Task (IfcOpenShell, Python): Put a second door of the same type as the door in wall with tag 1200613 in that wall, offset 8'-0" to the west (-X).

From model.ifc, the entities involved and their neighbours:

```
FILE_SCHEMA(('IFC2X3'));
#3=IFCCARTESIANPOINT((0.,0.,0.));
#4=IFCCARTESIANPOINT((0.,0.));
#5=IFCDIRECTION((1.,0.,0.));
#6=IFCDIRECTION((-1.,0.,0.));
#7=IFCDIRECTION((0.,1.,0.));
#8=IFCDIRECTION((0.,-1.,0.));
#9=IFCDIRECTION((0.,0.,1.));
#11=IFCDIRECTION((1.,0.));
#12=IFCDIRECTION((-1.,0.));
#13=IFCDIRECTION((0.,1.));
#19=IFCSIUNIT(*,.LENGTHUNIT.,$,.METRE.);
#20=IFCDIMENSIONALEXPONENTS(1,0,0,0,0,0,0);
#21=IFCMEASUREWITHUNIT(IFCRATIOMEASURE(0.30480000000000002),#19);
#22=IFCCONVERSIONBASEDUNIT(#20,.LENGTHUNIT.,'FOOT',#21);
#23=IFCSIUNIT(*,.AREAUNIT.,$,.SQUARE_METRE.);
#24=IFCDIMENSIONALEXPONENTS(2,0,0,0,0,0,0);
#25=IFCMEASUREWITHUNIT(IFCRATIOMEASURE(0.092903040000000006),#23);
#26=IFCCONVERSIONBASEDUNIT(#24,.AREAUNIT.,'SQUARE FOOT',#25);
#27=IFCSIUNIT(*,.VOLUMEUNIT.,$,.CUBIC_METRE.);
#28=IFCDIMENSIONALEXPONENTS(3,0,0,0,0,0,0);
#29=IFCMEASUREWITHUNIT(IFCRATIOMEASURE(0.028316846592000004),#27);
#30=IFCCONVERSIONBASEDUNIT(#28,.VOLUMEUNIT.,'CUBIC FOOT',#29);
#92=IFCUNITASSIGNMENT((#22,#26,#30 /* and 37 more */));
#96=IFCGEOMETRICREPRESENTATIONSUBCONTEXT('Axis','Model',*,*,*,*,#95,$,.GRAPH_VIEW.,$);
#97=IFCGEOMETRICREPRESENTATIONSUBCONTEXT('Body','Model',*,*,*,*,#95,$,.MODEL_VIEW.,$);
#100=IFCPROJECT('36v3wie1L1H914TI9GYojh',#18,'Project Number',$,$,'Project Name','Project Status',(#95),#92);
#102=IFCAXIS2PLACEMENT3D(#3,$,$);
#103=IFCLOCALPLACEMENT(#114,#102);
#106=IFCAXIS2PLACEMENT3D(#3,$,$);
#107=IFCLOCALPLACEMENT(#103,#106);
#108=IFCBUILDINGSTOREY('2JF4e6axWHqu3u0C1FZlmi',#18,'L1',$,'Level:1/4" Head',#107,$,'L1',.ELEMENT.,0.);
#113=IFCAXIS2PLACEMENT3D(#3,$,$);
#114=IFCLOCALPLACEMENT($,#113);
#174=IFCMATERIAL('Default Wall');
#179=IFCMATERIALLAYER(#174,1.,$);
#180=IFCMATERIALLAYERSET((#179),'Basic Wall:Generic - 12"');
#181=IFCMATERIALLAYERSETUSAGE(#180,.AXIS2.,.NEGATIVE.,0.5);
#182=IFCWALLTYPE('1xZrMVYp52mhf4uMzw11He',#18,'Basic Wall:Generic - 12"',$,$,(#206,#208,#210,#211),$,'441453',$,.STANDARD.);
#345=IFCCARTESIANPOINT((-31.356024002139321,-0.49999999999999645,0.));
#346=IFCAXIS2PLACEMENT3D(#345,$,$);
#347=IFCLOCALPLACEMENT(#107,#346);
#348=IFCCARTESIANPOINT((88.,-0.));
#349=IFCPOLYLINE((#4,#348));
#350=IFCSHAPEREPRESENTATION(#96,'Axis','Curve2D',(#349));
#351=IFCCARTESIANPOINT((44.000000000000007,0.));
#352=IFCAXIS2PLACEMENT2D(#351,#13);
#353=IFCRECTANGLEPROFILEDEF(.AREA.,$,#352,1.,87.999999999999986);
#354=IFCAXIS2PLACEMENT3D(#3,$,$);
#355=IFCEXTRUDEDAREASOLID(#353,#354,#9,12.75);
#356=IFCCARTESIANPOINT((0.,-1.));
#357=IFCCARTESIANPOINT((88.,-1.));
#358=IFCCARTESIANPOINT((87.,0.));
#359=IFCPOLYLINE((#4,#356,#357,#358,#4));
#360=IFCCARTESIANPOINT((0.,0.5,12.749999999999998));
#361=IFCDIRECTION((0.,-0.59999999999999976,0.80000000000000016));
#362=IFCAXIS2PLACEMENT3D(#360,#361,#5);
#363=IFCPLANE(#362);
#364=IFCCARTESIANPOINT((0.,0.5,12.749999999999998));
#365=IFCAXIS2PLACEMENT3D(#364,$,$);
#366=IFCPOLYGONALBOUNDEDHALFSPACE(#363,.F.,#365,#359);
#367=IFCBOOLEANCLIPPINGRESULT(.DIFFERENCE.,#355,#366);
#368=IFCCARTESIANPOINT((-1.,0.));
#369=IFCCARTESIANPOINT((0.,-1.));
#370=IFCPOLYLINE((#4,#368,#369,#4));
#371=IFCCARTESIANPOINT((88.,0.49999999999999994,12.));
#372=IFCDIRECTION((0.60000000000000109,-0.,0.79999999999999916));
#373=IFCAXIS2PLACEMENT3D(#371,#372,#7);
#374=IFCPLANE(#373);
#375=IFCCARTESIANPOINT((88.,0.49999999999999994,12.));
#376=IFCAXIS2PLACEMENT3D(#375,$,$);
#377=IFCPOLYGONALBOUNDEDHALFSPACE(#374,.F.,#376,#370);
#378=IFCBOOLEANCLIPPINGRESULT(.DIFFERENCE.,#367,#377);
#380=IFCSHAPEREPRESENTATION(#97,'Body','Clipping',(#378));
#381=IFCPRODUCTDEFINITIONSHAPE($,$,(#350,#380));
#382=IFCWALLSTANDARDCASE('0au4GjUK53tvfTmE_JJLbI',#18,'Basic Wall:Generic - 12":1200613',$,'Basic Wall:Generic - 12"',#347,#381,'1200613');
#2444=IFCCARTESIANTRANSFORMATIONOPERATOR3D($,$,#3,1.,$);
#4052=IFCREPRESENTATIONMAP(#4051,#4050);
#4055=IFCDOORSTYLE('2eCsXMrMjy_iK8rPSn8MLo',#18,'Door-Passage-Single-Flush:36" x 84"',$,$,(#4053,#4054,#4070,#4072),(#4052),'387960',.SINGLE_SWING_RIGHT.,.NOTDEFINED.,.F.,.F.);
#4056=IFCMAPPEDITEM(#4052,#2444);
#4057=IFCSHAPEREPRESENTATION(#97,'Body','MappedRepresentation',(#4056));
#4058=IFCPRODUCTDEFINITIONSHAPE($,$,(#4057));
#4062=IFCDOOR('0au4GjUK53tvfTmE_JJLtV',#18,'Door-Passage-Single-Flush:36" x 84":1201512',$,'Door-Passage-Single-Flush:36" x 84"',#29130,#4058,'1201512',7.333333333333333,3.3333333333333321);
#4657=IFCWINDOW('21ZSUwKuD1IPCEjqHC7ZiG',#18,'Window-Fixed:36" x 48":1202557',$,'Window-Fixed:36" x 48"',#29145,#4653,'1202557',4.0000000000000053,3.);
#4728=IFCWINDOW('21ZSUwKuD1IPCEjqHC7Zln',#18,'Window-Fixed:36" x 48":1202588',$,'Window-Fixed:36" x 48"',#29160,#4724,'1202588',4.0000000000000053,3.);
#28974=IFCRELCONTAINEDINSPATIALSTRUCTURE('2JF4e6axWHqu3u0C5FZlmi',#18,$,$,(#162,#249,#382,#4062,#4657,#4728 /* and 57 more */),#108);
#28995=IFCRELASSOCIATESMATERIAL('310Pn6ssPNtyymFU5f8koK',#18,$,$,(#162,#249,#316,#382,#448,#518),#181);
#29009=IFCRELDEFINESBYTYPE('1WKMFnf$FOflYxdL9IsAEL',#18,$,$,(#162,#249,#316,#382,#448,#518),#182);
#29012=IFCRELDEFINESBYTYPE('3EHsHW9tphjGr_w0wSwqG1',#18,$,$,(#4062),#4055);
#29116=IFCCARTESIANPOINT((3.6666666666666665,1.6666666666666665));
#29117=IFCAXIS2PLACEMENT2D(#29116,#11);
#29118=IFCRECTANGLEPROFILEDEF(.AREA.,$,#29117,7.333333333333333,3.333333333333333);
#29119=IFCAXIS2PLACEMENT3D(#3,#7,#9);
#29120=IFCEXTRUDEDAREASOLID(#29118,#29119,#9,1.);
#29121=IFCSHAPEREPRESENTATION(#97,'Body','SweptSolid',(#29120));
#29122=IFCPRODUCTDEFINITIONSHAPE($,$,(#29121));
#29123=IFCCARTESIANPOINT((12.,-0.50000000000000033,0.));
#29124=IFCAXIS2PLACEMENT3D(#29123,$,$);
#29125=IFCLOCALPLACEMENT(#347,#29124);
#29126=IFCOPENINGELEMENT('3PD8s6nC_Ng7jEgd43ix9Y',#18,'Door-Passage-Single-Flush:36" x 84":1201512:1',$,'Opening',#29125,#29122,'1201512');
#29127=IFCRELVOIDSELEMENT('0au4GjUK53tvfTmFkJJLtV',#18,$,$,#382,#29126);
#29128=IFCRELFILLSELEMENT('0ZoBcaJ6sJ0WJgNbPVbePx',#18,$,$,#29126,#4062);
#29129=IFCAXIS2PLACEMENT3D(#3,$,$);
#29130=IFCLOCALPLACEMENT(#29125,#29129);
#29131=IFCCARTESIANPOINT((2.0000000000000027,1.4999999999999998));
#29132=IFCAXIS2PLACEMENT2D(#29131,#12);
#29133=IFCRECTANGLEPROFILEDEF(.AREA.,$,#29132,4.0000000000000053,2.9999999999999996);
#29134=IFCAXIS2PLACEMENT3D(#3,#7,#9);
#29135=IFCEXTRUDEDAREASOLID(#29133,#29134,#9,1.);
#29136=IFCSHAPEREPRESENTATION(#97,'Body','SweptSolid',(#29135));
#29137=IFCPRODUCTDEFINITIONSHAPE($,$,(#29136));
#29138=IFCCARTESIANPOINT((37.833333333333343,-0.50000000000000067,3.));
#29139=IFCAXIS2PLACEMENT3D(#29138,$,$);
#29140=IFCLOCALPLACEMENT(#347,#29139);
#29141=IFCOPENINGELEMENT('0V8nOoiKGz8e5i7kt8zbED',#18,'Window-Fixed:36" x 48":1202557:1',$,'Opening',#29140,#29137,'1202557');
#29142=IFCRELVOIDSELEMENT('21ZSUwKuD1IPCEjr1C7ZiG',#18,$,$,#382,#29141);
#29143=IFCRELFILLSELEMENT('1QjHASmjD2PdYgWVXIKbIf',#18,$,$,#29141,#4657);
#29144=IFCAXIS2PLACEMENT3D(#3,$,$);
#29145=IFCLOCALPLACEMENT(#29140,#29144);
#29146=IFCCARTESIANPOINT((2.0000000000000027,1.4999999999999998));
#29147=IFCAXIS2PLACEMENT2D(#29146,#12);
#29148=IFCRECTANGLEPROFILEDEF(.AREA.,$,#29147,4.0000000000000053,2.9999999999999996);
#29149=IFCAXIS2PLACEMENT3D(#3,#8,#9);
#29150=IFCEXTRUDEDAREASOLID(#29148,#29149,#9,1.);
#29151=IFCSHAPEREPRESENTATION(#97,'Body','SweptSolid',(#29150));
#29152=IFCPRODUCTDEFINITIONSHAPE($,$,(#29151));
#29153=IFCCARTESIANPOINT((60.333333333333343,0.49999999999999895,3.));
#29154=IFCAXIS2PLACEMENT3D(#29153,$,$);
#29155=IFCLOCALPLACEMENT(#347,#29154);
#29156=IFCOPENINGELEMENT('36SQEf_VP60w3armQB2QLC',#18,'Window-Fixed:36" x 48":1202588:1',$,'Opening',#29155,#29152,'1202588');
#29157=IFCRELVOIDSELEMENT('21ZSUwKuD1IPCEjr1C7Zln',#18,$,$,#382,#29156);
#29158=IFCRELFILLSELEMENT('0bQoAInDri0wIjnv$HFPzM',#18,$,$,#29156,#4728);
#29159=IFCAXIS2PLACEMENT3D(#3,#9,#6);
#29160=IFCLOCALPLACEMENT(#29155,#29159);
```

```python
import ifcopenshell
import ifcopenshell.api.feature
import ifcopenshell.api.geometry
import ifcopenshell.api.root
import ifcopenshell.geom
import ifcopenshell.util.element
import ifcopenshell.util.placement
import ifcopenshell.util.shape
import ifcopenshell.util.unit

model = ifcopenshell.open("model.ifc")
unit_scale = ifcopenshell.util.unit.calculate_unit_scale(model)
settings = ifcopenshell.geom.settings()


def volume(element):
    """Net volume in cubic metres, openings subtracted."""
    shape = ifcopenshell.geom.create_shape(settings, element)
    return ifcopenshell.util.shape.get_volume(shape.geometry)


def reuse_history(source, copy):
    """copy_class also copies each property set's owner history, people and application; keep the originals."""
    for rel in copy.IsDefinedBy:
        if rel.is_a("IfcRelDefinesByProperties") and (history := rel.RelatingPropertyDefinition.OwnerHistory):
            rel.RelatingPropertyDefinition.OwnerHistory = source.OwnerHistory
            ifcopenshell.util.element.remove_deep2(model, history)


door = model.by_id(4062)
opening = door.FillsVoids[0].RelatingOpeningElement
wall = opening.VoidsElements[0].RelatingBuildingElement
before = volume(wall)
shift = ifcopenshell.util.placement.get_local_placement(wall.ObjectPlacement)[:3, 0] * -96 * 0.0254 / unit_scale

# copy_class copies the void relationship, type, container and properties, but no geometry.
new_opening = ifcopenshell.api.root.copy_class(model, product=opening)
new_opening.Representation = ifcopenshell.util.element.copy_deep(
    model, opening.Representation, exclude=["IfcGeometricRepresentationContext", "IfcRepresentationMap"]
)
new_opening.Name = 'Door-Passage-Single-Flush:36" x 84"'
new_opening.Tag = None
new_door = ifcopenshell.api.root.copy_class(model, product=door)
new_door.Representation = ifcopenshell.util.element.copy_deep(
    model, door.Representation, exclude=["IfcGeometricRepresentationContext", "IfcRepresentationMap"]
)
new_door.Name = 'Door-Passage-Single-Flush:36" x 84"'
new_door.Tag = None
reuse_history(door, new_door)
fills = ifcopenshell.api.feature.add_filling(model, opening=new_opening, element=new_door)
fills.OwnerHistory = new_door.OwnerHistory  # required in IFC2X3

for old, new in ((opening, new_opening), (door, new_door)):
    matrix = ifcopenshell.util.placement.get_local_placement(old.ObjectPlacement)
    matrix[:3, 3] += shift
    ifcopenshell.api.geometry.edit_object_placement(model, product=new, matrix=matrix, is_si=False)

after = volume(wall)

print(f"wall volume {before:.3f} -> {after:.3f} m3")

model.write("model-out.ifc")
```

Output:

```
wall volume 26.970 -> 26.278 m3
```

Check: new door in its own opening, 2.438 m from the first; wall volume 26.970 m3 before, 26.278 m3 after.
